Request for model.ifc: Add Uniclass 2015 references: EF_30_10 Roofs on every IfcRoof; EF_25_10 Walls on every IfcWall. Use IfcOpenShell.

First a look at what the model holds.

```python
import ifcopenshell

model = ifcopenshell.open("model.ifc")
print(model.schema)
print("classifications:", [c.Name for c in model.by_type("IfcClassification")])
for ifc_class in ("IfcDoor", "IfcRoof", "IfcStair", "IfcWall", "IfcWindow"):
    print(ifc_class, len(model.by_type(ifc_class)))
```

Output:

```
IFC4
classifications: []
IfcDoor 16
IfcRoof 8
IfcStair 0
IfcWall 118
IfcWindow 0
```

```python
import ifcopenshell
import ifcopenshell.api.classification

model = ifcopenshell.open("model.ifc")

system = ifcopenshell.api.classification.add_classification(model, classification="Uniclass 2015")

codes = {
    "IfcRoof": ("EF_30_10", "Roofs"),
    "IfcWall": ("EF_25_10", "Walls"),
}
for ifc_class, (code, name) in codes.items():
    products = model.by_type(ifc_class)
    ifcopenshell.api.classification.add_reference(
        model, products=products, classification=system, identification=code, name=name
    )
    print(code, len(products))

model.write("model-out.ifc")
```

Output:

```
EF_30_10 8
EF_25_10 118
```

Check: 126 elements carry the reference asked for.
